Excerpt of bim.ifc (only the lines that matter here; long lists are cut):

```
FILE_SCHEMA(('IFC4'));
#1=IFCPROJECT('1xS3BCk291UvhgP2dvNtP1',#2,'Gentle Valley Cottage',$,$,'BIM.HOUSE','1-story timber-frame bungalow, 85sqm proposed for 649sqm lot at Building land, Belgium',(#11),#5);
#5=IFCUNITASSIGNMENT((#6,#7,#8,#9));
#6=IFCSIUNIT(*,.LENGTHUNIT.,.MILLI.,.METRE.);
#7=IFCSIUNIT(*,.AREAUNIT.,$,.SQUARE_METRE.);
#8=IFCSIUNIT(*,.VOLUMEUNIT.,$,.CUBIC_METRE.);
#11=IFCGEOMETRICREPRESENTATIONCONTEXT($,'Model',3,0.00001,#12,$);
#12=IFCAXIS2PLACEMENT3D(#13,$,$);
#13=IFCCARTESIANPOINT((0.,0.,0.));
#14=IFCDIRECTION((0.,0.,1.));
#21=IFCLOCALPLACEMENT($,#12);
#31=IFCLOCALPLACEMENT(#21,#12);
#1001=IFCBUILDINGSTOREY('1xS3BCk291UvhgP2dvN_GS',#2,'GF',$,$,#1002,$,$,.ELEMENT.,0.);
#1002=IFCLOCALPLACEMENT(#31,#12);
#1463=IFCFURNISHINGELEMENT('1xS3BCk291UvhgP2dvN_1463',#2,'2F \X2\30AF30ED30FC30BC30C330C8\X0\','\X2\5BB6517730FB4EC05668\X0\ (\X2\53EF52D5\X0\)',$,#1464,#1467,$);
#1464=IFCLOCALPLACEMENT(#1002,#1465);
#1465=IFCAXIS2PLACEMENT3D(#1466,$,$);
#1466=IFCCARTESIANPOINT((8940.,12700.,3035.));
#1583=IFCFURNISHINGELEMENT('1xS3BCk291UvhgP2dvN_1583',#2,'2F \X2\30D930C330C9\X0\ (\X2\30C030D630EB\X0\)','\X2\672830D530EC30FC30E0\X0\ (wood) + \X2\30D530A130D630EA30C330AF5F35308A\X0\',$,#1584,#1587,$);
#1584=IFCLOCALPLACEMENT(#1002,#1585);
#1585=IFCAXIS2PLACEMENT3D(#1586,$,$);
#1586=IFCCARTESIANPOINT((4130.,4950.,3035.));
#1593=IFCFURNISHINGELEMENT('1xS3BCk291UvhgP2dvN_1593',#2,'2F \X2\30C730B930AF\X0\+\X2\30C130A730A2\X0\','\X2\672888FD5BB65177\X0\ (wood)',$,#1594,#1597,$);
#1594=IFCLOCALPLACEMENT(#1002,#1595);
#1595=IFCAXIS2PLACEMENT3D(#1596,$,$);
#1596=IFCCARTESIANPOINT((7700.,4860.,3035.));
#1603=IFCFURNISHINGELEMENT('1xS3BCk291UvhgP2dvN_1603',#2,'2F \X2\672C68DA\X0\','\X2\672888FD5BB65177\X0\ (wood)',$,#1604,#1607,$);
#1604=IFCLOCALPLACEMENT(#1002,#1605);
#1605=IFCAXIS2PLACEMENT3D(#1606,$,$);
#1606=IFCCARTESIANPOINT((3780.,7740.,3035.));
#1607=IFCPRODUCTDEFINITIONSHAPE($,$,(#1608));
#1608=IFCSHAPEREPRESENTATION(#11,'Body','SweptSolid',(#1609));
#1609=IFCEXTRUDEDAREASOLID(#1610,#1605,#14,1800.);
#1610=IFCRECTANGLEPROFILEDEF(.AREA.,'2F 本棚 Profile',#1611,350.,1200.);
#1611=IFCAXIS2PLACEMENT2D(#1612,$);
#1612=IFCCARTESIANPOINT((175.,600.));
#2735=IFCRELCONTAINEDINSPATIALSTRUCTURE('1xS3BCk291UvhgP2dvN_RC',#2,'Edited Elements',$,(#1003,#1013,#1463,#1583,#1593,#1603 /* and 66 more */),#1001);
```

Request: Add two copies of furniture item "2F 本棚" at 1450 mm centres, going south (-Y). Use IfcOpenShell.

```python
import numpy as np
import ifcopenshell
import ifcopenshell.api.geometry
import ifcopenshell.api.root
import ifcopenshell.util.element
import ifcopenshell.util.placement
import ifcopenshell.util.unit

model = ifcopenshell.open("bim.ifc")
unit_scale = ifcopenshell.util.unit.calculate_unit_scale(model)


def reuse_history(source, copy):
    """copy_class also copies each property set's owner history, people and application; keep the originals."""
    for rel in copy.IsDefinedBy:
        if rel.is_a("IfcRelDefinesByProperties") and (history := rel.RelatingPropertyDefinition.OwnerHistory):
            rel.RelatingPropertyDefinition.OwnerHistory = source.OwnerHistory
            ifcopenshell.util.element.remove_deep2(model, history)


source = model.by_guid("1xS3BCk291UvhgP2dvN_1603")
base = ifcopenshell.util.placement.get_local_placement(source.ObjectPlacement)
step = np.array([0.0, -1.0, 0.0]) * 1.45 / unit_scale

for i in range(1, 3):
    copy = ifcopenshell.api.root.copy_class(model, product=source)
    copy.Representation = ifcopenshell.util.element.copy_deep(
        model, source.Representation, exclude=["IfcGeometricRepresentationContext", "IfcRepresentationMap"]
    )
    reuse_history(source, copy)
    matrix = base.copy()
    matrix[:3, 3] += i * step
    print("added at", matrix[:3, 3].round(3) + 0.0)
    ifcopenshell.api.geometry.edit_object_placement(model, product=copy, matrix=matrix, is_si=False)

model.write("bim_rev.ifc")
```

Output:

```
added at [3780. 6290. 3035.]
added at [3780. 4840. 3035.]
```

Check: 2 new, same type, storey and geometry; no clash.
